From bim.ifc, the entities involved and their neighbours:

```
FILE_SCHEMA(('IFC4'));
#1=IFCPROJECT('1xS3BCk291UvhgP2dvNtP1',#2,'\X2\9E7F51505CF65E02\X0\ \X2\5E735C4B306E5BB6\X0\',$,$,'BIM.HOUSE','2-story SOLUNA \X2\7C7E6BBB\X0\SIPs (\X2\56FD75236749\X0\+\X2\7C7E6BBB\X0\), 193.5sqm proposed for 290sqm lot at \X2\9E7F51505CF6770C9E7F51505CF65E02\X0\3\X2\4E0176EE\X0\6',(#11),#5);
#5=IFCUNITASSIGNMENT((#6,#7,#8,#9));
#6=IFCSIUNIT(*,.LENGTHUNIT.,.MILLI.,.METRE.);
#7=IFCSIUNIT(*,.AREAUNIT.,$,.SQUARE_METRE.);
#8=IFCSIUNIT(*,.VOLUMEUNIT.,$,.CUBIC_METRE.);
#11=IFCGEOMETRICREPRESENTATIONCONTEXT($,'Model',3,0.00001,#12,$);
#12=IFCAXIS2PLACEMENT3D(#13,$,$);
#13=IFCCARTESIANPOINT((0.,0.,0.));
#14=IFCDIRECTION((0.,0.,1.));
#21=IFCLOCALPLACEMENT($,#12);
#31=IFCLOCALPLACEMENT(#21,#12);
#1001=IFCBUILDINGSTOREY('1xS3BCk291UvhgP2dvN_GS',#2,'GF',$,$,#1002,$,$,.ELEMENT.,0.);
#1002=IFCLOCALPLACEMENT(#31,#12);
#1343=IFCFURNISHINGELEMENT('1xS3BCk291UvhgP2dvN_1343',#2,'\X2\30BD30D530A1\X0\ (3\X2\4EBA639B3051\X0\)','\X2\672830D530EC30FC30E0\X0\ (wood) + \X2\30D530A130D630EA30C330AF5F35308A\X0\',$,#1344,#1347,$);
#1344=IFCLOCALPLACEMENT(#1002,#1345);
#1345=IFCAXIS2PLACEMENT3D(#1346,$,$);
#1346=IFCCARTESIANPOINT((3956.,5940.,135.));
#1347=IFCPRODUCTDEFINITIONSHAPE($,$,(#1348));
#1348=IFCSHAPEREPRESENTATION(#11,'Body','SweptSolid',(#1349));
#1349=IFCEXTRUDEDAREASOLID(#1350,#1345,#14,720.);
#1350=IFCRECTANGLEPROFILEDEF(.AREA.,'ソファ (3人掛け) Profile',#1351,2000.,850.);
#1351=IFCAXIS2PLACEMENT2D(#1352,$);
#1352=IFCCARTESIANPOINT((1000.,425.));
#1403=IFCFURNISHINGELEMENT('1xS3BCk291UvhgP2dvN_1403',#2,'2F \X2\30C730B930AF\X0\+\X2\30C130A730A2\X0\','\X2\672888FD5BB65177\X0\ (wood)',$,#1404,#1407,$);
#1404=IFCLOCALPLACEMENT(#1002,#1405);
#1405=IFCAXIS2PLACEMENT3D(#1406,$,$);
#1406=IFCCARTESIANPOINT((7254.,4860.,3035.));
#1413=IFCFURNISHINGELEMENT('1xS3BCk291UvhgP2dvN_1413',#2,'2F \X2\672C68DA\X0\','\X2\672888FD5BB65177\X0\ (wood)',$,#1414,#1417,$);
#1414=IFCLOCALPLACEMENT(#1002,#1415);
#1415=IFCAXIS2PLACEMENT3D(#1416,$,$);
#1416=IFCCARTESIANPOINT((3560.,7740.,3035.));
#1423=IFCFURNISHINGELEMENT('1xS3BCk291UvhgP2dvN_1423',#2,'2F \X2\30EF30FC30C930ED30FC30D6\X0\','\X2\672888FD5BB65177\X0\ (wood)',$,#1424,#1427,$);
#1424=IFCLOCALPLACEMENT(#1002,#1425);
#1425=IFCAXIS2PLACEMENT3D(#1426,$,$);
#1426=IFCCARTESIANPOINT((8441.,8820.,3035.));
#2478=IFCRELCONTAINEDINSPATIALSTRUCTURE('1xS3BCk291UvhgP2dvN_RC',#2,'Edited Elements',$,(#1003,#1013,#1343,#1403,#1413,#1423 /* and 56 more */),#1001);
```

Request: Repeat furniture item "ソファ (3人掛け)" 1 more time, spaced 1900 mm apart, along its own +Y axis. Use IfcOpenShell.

```python
import ifcopenshell
import ifcopenshell.api.geometry
import ifcopenshell.api.root
import ifcopenshell.util.element
import ifcopenshell.util.placement

model = ifcopenshell.open("bim.ifc")


def reuse_history(source, copy):
    """copy_class also copies each property set's owner history, people and application; keep the originals."""
    for rel in copy.IsDefinedBy:
        if rel.is_a("IfcRelDefinesByProperties") and (history := rel.RelatingPropertyDefinition.OwnerHistory):
            rel.RelatingPropertyDefinition.OwnerHistory = source.OwnerHistory
            ifcopenshell.util.element.remove_deep2(model, history)


source = model.by_guid("1xS3BCk291UvhgP2dvN_1343")
base = ifcopenshell.util.placement.get_local_placement(source.ObjectPlacement)
step = base[:3, 1] * 1900.0

for i in range(1, 2):
    copy = ifcopenshell.api.root.copy_class(model, product=source)
    copy.Representation = ifcopenshell.util.element.copy_deep(
        model, source.Representation, exclude=["IfcGeometricRepresentationContext", "IfcRepresentationMap"]
    )
    reuse_history(source, copy)
    matrix = base.copy()
    matrix[:3, 3] += i * step
    print("added at", matrix[:3, 3].round(3) + 0.0)
    ifcopenshell.api.geometry.edit_object_placement(model, product=copy, matrix=matrix, is_si=False)

model.write("bim-out.ifc")
```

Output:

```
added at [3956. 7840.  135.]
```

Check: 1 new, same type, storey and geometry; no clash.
